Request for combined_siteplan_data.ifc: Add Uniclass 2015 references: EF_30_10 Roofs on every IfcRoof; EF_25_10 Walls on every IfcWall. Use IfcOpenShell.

First a look at what the model holds.

```python
import ifcopenshell

model = ifcopenshell.open("combined_siteplan_data.ifc")
print(model.schema)
print("classifications:", [c.Name for c in model.by_type("IfcClassification")])
for ifc_class in ("IfcDoor", "IfcRoof", "IfcStair", "IfcWall", "IfcWindow"):
    print(ifc_class, len(model.by_type(ifc_class)))
```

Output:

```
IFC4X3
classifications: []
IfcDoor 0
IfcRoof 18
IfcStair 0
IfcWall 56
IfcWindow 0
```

```python
import ifcopenshell
import ifcopenshell.api.classification

model = ifcopenshell.open("combined_siteplan_data.ifc")

system = ifcopenshell.api.classification.add_classification(model, classification="Uniclass 2015")

codes = {
    "IfcRoof": ("EF_30_10", "Roofs"),
    "IfcWall": ("EF_25_10", "Walls"),
}
for ifc_class, (code, name) in codes.items():
    products = model.by_type(ifc_class)
    ifcopenshell.api.classification.add_reference(
        model, products=products, classification=system, identification=code, name=name
    )
    print(code, len(products))

model.write("combined_siteplan_data_v2.ifc")
```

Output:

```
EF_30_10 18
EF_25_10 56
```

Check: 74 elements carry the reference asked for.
